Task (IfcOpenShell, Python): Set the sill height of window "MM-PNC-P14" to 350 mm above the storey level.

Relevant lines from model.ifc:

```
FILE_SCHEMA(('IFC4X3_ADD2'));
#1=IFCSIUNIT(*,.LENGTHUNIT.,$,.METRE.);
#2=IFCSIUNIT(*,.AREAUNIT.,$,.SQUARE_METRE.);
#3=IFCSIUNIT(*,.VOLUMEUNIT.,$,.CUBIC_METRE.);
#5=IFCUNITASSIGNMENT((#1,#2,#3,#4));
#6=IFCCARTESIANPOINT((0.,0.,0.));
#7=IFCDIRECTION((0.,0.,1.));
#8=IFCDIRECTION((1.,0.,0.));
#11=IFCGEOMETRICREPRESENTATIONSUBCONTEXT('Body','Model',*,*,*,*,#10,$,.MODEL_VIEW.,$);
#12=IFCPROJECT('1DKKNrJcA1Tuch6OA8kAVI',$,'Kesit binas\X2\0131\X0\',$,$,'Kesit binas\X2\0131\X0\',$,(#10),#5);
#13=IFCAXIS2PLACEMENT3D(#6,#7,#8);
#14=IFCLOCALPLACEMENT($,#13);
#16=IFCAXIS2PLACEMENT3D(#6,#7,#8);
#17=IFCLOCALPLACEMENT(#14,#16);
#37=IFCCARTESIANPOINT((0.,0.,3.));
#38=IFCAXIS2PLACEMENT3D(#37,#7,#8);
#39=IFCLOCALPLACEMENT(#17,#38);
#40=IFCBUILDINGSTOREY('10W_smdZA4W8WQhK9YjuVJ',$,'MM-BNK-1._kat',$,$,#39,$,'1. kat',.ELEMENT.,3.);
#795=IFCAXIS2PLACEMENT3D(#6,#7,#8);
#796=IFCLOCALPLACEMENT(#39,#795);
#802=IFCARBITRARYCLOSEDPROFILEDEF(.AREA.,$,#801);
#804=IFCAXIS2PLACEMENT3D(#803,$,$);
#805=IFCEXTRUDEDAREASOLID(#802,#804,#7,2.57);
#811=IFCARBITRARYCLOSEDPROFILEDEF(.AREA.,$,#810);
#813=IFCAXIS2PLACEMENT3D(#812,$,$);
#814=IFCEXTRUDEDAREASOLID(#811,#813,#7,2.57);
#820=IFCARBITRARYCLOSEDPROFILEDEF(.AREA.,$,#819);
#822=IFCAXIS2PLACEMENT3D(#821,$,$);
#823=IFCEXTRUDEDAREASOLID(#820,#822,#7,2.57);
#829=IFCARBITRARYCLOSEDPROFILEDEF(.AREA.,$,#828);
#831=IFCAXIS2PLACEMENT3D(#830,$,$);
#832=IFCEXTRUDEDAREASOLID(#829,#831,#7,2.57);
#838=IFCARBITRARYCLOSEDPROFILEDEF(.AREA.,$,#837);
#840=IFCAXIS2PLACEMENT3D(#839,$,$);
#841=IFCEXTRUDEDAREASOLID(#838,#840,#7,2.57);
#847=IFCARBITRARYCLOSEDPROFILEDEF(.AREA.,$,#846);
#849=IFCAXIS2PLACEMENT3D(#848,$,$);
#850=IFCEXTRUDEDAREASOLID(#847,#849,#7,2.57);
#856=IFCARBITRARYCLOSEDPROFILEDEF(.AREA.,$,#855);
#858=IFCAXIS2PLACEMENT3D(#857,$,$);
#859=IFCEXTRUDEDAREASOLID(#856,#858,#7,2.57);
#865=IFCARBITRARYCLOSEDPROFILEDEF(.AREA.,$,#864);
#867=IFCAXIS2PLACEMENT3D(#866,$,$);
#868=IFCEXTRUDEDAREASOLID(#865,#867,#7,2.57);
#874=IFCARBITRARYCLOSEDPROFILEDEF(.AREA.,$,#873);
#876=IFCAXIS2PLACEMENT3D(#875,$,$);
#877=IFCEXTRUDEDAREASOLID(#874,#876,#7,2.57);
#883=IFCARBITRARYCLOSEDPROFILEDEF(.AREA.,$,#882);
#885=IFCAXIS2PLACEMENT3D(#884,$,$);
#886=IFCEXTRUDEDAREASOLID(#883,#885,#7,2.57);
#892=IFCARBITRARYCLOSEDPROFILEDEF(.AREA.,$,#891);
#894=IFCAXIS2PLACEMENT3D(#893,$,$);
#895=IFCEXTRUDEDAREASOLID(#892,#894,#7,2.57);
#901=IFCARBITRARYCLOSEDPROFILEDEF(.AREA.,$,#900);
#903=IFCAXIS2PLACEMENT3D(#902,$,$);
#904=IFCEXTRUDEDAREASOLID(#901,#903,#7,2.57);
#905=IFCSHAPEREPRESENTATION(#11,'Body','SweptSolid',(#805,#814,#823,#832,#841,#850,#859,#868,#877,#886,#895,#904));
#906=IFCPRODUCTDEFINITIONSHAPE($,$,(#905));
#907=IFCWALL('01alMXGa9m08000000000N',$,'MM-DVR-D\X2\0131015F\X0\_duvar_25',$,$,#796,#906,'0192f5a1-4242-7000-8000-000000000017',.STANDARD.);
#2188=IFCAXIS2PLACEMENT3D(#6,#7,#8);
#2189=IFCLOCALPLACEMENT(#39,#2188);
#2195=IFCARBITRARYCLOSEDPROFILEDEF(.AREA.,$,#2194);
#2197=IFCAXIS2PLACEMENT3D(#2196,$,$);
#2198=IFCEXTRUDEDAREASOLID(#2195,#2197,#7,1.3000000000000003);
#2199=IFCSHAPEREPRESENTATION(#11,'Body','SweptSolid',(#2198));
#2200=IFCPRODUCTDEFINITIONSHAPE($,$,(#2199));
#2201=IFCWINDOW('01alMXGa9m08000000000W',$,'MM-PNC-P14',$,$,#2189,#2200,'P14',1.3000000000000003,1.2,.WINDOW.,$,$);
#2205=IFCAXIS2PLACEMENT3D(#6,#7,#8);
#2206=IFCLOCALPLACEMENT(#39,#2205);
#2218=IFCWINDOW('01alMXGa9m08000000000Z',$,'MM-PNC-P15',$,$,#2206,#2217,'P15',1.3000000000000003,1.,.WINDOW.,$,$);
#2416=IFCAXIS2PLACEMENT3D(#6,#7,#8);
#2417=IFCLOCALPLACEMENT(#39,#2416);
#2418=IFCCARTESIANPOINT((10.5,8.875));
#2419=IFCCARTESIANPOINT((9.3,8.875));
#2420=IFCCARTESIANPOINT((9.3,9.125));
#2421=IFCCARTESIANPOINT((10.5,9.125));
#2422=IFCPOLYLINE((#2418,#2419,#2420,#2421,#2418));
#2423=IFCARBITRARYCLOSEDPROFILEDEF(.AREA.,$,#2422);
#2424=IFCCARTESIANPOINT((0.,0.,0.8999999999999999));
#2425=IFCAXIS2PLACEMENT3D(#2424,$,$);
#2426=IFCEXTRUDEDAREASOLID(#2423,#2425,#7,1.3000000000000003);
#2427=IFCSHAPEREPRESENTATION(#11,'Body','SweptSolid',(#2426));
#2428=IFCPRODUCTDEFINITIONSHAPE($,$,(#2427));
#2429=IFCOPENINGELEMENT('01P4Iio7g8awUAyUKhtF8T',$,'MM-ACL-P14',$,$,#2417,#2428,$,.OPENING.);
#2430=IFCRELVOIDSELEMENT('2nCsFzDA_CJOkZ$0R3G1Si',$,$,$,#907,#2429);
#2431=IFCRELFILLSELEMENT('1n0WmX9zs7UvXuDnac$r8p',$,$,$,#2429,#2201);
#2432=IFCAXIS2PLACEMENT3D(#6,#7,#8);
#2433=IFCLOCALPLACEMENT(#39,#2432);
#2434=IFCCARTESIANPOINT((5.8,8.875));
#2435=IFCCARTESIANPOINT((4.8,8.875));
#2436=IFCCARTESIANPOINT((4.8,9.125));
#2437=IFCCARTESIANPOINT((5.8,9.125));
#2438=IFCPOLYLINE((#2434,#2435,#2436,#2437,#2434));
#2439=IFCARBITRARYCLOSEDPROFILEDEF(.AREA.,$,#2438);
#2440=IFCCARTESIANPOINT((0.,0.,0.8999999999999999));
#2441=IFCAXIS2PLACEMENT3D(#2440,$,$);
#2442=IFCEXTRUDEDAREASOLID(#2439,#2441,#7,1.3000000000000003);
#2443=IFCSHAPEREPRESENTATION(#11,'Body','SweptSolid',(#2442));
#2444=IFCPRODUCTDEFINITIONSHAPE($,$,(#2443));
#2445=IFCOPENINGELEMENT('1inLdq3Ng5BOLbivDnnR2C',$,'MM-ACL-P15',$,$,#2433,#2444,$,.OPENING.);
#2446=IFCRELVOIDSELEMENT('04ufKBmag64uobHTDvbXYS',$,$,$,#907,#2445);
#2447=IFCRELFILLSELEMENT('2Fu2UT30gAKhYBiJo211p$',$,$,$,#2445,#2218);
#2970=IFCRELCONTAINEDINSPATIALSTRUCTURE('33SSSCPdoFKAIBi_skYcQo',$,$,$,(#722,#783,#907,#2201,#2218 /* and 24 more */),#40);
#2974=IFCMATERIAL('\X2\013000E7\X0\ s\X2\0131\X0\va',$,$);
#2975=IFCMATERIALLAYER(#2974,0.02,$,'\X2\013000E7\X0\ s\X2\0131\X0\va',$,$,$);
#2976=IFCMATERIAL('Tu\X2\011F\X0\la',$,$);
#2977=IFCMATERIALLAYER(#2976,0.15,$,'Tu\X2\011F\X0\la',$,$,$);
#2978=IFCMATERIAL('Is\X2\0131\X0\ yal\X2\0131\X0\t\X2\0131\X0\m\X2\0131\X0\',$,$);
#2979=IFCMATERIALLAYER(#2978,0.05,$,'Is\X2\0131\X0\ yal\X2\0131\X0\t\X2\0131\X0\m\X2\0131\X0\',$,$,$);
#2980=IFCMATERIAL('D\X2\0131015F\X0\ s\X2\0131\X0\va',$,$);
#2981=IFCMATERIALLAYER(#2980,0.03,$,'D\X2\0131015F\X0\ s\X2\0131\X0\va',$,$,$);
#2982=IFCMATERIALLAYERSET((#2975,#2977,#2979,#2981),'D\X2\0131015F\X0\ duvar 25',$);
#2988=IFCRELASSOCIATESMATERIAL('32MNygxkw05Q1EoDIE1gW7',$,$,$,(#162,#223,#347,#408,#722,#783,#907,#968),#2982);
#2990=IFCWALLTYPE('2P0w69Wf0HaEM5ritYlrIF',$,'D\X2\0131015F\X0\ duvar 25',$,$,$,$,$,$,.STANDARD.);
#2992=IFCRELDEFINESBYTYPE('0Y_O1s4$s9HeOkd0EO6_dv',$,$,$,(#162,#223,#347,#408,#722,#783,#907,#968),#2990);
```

```python
import numpy as np
import ifcopenshell
import ifcopenshell.api.geometry
import ifcopenshell.geom
import ifcopenshell.util.element
import ifcopenshell.util.placement
import ifcopenshell.util.shape
import ifcopenshell.util.unit

model = ifcopenshell.open("model.ifc")
unit_scale = ifcopenshell.util.unit.calculate_unit_scale(model)

window = model.by_id(2201)
opening = window.FillsVoids[0].RelatingOpeningElement
storey = ifcopenshell.util.element.get_container(window, ifc_class="IfcBuildingStorey")
level = ifcopenshell.util.placement.get_local_placement(storey.ObjectPlacement)[2, 3]

# The opening's origin need not be at the sill, so measure its lowest point.
shape = ifcopenshell.geom.create_shape(ifcopenshell.geom.settings(), opening)
bottom = ifcopenshell.util.shape.get_shape_bottom_elevation(shape, shape.geometry) / unit_scale
dz = level + 0.35 - bottom

shift = np.array([0.0, 0.0, dz])
# The window is not placed relative to its opening, so move both.
for product in (opening, window):
    matrix = ifcopenshell.util.placement.get_local_placement(product.ObjectPlacement)
    matrix[:3, 3] += shift
    ifcopenshell.api.geometry.edit_object_placement(model, product=product, matrix=matrix, is_si=False)

print(f"moved by {dz * unit_scale:+.3f} m")

model.write("model_updated.ifc")
```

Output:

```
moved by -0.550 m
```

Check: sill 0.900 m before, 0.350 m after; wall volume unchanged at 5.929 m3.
